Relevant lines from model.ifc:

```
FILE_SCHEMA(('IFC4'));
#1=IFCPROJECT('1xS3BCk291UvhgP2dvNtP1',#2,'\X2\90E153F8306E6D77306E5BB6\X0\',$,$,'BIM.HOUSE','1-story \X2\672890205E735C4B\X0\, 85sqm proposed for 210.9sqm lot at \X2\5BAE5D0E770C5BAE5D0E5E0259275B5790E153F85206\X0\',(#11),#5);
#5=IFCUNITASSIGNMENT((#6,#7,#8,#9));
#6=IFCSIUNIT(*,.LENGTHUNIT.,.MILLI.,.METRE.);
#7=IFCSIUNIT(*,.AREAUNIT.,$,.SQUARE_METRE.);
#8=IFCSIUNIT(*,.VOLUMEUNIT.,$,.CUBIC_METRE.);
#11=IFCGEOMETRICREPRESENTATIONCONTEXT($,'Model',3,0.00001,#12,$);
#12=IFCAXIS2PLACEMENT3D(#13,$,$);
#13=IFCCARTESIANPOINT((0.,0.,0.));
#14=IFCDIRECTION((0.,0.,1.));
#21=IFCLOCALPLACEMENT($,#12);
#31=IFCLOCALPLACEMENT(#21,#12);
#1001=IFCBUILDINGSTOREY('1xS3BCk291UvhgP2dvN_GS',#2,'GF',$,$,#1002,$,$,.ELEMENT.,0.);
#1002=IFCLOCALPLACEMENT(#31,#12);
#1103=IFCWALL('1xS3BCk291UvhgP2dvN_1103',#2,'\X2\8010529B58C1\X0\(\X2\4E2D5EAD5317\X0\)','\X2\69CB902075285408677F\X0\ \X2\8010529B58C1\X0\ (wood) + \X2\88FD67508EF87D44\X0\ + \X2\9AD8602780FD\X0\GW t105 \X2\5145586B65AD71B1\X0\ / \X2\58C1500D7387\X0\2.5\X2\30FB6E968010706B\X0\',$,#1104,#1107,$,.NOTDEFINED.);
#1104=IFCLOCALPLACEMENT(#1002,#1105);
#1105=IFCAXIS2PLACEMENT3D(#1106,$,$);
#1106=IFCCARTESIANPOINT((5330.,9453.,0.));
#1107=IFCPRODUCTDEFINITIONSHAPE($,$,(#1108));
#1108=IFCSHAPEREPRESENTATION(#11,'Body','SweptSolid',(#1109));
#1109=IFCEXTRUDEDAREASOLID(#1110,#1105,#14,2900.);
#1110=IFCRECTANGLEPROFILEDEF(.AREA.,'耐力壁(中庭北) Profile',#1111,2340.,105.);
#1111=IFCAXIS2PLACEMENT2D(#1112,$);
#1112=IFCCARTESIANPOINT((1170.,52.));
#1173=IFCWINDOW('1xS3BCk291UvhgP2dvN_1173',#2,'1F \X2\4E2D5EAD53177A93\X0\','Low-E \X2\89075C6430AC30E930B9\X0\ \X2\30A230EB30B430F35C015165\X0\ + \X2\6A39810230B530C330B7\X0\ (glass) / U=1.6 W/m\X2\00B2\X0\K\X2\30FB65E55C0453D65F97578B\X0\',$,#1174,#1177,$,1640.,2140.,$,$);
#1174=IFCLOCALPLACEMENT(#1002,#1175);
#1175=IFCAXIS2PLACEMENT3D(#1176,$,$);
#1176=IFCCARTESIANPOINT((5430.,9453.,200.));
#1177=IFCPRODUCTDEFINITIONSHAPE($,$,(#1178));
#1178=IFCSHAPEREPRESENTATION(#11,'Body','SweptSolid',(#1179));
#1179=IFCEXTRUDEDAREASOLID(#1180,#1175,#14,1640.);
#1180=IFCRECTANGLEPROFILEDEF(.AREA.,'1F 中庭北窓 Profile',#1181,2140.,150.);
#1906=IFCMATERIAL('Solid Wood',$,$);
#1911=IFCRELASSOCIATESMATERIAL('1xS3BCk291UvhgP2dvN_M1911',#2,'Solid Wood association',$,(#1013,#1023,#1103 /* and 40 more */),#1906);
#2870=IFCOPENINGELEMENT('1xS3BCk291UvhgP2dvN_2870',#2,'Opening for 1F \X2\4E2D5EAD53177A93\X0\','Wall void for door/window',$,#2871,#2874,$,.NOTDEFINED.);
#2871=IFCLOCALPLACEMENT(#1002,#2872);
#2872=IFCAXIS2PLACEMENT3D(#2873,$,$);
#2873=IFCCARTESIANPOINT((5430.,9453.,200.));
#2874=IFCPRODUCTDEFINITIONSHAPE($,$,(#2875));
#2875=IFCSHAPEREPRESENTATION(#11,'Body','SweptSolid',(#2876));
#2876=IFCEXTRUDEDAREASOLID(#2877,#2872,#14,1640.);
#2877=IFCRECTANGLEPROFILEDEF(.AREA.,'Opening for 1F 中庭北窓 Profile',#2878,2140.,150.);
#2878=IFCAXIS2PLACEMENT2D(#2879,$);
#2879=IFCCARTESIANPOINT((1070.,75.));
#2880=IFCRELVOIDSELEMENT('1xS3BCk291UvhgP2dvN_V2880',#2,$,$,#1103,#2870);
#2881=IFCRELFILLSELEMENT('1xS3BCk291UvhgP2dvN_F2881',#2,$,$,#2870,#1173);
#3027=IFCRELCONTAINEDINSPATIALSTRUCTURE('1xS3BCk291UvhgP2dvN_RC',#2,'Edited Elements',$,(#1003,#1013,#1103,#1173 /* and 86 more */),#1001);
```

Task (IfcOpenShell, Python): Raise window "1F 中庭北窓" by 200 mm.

```python
import numpy as np
import ifcopenshell
import ifcopenshell.api.geometry
import ifcopenshell.util.placement
import ifcopenshell.util.unit

model = ifcopenshell.open("model.ifc")
unit_scale = ifcopenshell.util.unit.calculate_unit_scale(model)

window = model.by_guid("1xS3BCk291UvhgP2dvN_1173")
opening = window.FillsVoids[0].RelatingOpeningElement
dz = 0.2 / unit_scale

shift = np.array([0.0, 0.0, dz])
# The window is not placed relative to its opening, so move both.
for product in (opening, window):
    matrix = ifcopenshell.util.placement.get_local_placement(product.ObjectPlacement)
    matrix[:3, 3] += shift
    ifcopenshell.api.geometry.edit_object_placement(model, product=product, matrix=matrix, is_si=False)

print(f"moved by {dz * unit_scale:+.3f} m")

model.write("model_updated.ifc")
```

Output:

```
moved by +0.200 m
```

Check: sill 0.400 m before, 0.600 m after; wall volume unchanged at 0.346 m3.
